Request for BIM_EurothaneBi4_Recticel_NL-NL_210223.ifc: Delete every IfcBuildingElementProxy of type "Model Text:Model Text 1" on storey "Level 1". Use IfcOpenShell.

First a look at what the model holds.

```python
import ifcopenshell
import ifcopenshell.util.element

model = ifcopenshell.open("BIM_EurothaneBi4_Recticel_NL-NL_210223.ifc")
print(model.schema)
storey = next(s for s in model.by_type("IfcBuildingStorey") if s.Name == "Level 1")
proxies = [e for e in ifcopenshell.util.element.get_decomposition(storey) if e.is_a("IfcBuildingElementProxy")]
seen = {}
for e in proxies:
    element_type = ifcopenshell.util.element.get_type(e)
    name = element_type.Name if element_type not in (None, e) else None
    seen[name] = seen.get(name, 0) + 1
for name, count in sorted(seen.items(), key=str):
    print(count, "x", name)
```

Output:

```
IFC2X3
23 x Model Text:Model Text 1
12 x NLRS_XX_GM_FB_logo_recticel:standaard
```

```python
import ifcopenshell
import ifcopenshell.api.root
import ifcopenshell.util.element

model = ifcopenshell.open("BIM_EurothaneBi4_Recticel_NL-NL_210223.ifc")

storey = next(s for s in model.by_type("IfcBuildingStorey") if s.Name == "Level 1")
proxies = [e for e in ifcopenshell.util.element.get_decomposition(storey) if e.is_a("IfcBuildingElementProxy")]
targets = [e for e in proxies if (t := ifcopenshell.util.element.get_type(e)) not in (None, e) and t.Name == "Model Text:Model Text 1"]

for e in targets:
    ifcopenshell.api.root.remove_product(model, product=e)
print(len(targets), "removed")

model.write("BIM_EurothaneBi4_Recticel_NL-NL_210223_rev.ifc")
```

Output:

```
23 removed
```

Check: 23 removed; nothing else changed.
